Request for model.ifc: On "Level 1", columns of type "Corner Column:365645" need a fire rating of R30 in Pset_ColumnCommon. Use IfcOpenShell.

First a look at what the model holds.

```python
import ifcopenshell
import ifcopenshell.util.element

model = ifcopenshell.open("model.ifc")
print(model.schema)
storey = next(s for s in model.by_type("IfcBuildingStorey") if s.Name == "Level 1")
columns = [e for e in ifcopenshell.util.element.get_decomposition(storey) if e.is_a("IfcColumn")]
seen = {}
for e in columns:
    element_type = ifcopenshell.util.element.get_type(e)
    key = (element_type.Name if element_type != e and element_type else None, ifcopenshell.util.element.get_pset(e, "Pset_ColumnCommon", "FireRating"))
    seen[key] = seen.get(key, 0) + 1
for (name, value), count in sorted(seen.items(), key=str):
    print(count, "x", name, "|", value)
```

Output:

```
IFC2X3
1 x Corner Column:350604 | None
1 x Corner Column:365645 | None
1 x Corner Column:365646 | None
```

```python
import ifcopenshell
import ifcopenshell.api.pset
import ifcopenshell.util.element

model = ifcopenshell.open("model.ifc")

storey = next(s for s in model.by_type("IfcBuildingStorey") if s.Name == "Level 1")
columns = [e for e in ifcopenshell.util.element.get_decomposition(storey) if e.is_a("IfcColumn")]

count = 0
for e in columns:
    element_type = ifcopenshell.util.element.get_type(e)
    if element_type in (None, e) or element_type.Name != "Corner Column:365645":
        continue
    # add_pset returns the element's existing set when there is one.
    pset = ifcopenshell.api.pset.add_pset(model, product=e, name="Pset_ColumnCommon")
    ifcopenshell.api.pset.edit_pset(model, pset=pset, properties={"FireRating": "R30"})
    count += 1

print(count, "columns updated")

model.write("model-out.ifc")
```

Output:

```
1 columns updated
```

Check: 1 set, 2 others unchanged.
